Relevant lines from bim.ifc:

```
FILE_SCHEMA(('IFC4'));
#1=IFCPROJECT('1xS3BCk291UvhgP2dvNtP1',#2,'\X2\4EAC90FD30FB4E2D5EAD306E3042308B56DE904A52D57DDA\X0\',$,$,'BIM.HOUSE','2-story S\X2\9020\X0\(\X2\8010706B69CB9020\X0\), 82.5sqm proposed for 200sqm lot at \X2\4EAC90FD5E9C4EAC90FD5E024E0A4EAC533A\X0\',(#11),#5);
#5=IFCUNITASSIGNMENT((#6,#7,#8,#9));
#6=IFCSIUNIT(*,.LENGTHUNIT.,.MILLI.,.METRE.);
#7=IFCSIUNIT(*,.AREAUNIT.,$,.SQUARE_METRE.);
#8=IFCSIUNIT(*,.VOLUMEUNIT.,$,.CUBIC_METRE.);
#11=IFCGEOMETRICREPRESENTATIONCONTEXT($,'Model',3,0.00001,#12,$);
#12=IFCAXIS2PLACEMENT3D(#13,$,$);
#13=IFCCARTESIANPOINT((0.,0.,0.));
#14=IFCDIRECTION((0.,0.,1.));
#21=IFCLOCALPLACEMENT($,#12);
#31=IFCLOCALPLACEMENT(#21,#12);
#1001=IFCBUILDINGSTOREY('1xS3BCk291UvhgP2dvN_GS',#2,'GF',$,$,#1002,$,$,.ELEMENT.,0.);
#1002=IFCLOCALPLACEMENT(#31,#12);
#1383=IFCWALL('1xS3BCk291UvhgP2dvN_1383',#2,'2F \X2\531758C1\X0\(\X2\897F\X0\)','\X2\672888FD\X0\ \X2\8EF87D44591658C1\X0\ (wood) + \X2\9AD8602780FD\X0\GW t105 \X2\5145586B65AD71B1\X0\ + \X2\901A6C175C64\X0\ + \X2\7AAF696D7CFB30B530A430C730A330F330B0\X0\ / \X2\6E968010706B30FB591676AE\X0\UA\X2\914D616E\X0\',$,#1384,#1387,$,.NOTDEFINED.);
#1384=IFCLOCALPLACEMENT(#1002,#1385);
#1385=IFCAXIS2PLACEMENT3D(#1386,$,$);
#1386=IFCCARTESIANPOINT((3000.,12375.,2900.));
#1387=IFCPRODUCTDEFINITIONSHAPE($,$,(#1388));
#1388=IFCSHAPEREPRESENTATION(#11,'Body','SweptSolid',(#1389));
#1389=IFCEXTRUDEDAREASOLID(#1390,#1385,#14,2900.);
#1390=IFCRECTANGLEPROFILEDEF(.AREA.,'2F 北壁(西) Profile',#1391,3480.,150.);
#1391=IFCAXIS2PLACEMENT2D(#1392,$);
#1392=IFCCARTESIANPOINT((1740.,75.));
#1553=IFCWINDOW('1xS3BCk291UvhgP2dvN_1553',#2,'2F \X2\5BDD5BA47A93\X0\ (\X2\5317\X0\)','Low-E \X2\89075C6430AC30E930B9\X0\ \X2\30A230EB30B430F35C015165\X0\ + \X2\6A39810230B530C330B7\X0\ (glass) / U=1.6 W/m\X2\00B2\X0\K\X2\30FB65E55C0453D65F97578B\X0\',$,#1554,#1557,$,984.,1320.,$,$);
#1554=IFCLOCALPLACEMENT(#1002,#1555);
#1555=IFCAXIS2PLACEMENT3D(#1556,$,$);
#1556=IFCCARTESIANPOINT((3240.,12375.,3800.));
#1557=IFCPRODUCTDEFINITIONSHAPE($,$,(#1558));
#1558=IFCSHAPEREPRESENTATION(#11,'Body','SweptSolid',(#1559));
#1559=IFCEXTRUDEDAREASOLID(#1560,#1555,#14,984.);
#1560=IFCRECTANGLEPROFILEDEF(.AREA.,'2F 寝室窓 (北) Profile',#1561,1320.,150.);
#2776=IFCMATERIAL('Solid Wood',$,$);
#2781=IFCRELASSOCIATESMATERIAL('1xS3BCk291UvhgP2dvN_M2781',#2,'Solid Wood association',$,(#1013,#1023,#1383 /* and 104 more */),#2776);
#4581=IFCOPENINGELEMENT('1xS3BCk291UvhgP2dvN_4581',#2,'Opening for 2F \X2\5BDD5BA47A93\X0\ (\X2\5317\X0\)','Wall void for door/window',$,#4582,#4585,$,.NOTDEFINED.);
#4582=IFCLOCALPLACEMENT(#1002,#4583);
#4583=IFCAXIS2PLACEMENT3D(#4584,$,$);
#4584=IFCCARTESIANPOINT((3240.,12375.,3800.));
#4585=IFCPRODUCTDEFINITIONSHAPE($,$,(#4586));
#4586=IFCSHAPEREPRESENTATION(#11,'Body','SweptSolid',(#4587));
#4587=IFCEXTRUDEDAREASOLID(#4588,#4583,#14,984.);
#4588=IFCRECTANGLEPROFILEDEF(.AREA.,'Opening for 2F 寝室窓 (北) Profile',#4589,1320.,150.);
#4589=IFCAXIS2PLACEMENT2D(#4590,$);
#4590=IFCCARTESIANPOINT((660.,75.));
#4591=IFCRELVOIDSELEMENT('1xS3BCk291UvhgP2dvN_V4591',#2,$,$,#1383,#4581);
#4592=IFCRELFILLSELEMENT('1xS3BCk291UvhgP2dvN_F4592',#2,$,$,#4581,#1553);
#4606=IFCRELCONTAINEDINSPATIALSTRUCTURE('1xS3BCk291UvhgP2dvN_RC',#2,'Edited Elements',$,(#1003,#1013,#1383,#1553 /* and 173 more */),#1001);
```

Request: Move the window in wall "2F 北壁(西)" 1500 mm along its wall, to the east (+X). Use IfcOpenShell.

```python
import ifcopenshell
import ifcopenshell.api.geometry
import ifcopenshell.util.placement
import ifcopenshell.util.unit

model = ifcopenshell.open("bim.ifc")
unit_scale = ifcopenshell.util.unit.calculate_unit_scale(model)

window = model.by_id(1553)
opening = window.FillsVoids[0].RelatingOpeningElement
wall = opening.VoidsElements[0].RelatingBuildingElement

wall_matrix = ifcopenshell.util.placement.get_local_placement(wall.ObjectPlacement)
shift = wall_matrix[:3, 0] * 1.5 / unit_scale
before = ifcopenshell.util.placement.get_local_placement(window.ObjectPlacement)[:3, 3].copy()

# The window is not placed relative to its opening, so move both.
for product in (opening, window):
    matrix = ifcopenshell.util.placement.get_local_placement(product.ObjectPlacement)
    matrix[:3, 3] += shift
    ifcopenshell.api.geometry.edit_object_placement(model, product=product, matrix=matrix, is_si=False)

after = ifcopenshell.util.placement.get_local_placement(window.ObjectPlacement)[:3, 3]
print("window moved by", (after - before).round(3) + 0.0)

model.write("bim_rev.ifc")
```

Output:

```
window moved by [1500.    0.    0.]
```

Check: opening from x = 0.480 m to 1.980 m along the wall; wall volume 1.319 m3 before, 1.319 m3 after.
